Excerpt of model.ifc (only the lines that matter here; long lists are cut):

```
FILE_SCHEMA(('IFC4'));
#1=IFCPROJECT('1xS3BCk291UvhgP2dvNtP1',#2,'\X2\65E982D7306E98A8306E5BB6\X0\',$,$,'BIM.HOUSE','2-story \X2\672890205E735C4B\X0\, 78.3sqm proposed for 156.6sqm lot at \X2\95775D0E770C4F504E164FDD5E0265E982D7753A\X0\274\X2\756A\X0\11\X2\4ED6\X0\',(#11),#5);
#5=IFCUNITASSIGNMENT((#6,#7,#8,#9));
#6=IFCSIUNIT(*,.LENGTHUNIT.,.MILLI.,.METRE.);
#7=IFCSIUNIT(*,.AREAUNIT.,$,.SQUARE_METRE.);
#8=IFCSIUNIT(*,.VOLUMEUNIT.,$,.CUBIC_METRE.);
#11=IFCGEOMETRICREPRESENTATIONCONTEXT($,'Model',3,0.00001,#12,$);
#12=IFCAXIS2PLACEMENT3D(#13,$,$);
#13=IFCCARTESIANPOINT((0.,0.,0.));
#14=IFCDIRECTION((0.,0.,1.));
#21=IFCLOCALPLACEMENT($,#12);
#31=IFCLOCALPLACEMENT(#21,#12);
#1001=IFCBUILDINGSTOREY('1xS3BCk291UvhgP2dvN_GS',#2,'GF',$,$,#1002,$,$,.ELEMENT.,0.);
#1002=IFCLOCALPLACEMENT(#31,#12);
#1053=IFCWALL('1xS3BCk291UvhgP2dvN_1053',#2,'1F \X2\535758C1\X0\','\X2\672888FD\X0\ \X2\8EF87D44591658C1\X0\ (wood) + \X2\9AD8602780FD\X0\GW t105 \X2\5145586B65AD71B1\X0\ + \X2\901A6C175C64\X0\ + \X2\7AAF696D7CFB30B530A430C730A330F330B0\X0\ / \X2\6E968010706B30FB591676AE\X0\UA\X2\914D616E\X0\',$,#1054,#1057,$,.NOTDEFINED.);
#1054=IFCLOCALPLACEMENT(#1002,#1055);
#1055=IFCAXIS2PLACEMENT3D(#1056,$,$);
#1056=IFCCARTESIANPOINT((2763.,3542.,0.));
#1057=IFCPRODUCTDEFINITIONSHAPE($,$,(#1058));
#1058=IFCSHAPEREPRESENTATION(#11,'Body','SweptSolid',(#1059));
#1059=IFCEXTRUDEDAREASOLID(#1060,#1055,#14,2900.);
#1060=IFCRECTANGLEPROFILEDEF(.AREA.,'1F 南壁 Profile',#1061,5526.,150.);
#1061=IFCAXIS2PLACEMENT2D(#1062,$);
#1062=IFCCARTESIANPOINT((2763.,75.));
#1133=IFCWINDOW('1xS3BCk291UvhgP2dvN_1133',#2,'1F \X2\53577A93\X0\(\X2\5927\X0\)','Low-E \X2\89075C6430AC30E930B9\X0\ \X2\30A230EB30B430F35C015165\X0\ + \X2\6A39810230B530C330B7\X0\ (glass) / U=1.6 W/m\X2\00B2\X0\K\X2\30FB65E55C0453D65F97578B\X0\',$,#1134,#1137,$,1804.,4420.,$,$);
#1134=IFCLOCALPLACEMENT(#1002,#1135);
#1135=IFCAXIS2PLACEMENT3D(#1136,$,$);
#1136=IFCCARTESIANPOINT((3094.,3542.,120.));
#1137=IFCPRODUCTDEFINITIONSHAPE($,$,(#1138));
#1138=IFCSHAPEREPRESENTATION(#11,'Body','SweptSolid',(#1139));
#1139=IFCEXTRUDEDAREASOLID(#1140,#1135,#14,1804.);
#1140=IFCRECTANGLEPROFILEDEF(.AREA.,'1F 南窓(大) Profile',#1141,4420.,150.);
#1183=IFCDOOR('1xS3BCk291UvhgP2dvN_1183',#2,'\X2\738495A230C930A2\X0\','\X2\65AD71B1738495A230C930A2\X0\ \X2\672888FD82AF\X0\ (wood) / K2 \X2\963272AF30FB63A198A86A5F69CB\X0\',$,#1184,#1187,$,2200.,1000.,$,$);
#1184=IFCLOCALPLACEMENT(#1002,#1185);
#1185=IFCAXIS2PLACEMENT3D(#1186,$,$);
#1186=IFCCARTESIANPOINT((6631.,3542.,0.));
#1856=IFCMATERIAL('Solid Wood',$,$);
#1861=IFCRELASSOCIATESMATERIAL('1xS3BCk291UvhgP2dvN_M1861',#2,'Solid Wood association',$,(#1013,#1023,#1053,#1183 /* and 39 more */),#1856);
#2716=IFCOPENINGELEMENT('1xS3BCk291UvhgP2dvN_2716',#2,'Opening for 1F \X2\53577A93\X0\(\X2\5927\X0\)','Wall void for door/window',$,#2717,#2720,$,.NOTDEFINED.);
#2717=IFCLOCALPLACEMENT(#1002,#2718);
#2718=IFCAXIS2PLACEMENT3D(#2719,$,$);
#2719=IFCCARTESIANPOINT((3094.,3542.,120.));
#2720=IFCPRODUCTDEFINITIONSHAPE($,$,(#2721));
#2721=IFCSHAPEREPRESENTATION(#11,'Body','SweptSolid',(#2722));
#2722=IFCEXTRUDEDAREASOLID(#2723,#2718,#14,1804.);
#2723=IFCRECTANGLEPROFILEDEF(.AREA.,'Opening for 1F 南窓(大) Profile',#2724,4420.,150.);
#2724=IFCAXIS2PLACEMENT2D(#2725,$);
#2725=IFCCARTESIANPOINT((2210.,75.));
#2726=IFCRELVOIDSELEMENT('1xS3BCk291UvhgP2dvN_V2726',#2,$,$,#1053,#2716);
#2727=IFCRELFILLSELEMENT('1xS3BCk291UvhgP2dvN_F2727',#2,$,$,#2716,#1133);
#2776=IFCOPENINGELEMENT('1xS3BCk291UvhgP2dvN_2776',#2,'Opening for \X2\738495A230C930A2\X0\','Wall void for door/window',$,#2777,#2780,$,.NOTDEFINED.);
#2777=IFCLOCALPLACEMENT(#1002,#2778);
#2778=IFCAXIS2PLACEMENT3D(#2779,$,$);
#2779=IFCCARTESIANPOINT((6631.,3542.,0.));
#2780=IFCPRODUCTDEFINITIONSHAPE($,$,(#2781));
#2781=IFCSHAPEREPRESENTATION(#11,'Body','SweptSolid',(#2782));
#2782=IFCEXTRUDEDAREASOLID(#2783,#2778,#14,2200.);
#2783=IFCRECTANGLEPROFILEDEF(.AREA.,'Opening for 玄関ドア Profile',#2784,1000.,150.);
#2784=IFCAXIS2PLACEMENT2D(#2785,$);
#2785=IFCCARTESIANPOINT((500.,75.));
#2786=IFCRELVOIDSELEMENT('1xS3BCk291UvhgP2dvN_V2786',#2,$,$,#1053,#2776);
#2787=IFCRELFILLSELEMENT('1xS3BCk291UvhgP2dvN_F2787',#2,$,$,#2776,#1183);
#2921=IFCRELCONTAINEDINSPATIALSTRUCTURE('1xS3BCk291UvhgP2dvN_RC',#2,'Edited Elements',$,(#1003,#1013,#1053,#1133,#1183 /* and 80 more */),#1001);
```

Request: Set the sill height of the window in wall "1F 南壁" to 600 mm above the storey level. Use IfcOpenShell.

```python
import numpy as np
import ifcopenshell
import ifcopenshell.api.geometry
import ifcopenshell.geom
import ifcopenshell.util.element
import ifcopenshell.util.placement
import ifcopenshell.util.shape
import ifcopenshell.util.unit

model = ifcopenshell.open("model.ifc")
unit_scale = ifcopenshell.util.unit.calculate_unit_scale(model)

window = model.by_guid("1xS3BCk291UvhgP2dvN_1133")
opening = window.FillsVoids[0].RelatingOpeningElement
storey = ifcopenshell.util.element.get_container(window, ifc_class="IfcBuildingStorey")
level = ifcopenshell.util.placement.get_local_placement(storey.ObjectPlacement)[2, 3]

# The opening's origin need not be at the sill, so measure its lowest point.
shape = ifcopenshell.geom.create_shape(ifcopenshell.geom.settings(), opening)
bottom = ifcopenshell.util.shape.get_shape_bottom_elevation(shape, shape.geometry) / unit_scale
dz = level + 0.6 / unit_scale - bottom

shift = np.array([0.0, 0.0, dz])
# The window is not placed relative to its opening, so move both.
for product in (opening, window):
    matrix = ifcopenshell.util.placement.get_local_placement(product.ObjectPlacement)
    matrix[:3, 3] += shift
    ifcopenshell.api.geometry.edit_object_placement(model, product=product, matrix=matrix, is_si=False)

print(f"moved by {dz * unit_scale:+.3f} m")

model.write("model_rev.ifc")
```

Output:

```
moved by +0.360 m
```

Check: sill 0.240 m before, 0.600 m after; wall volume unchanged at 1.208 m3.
